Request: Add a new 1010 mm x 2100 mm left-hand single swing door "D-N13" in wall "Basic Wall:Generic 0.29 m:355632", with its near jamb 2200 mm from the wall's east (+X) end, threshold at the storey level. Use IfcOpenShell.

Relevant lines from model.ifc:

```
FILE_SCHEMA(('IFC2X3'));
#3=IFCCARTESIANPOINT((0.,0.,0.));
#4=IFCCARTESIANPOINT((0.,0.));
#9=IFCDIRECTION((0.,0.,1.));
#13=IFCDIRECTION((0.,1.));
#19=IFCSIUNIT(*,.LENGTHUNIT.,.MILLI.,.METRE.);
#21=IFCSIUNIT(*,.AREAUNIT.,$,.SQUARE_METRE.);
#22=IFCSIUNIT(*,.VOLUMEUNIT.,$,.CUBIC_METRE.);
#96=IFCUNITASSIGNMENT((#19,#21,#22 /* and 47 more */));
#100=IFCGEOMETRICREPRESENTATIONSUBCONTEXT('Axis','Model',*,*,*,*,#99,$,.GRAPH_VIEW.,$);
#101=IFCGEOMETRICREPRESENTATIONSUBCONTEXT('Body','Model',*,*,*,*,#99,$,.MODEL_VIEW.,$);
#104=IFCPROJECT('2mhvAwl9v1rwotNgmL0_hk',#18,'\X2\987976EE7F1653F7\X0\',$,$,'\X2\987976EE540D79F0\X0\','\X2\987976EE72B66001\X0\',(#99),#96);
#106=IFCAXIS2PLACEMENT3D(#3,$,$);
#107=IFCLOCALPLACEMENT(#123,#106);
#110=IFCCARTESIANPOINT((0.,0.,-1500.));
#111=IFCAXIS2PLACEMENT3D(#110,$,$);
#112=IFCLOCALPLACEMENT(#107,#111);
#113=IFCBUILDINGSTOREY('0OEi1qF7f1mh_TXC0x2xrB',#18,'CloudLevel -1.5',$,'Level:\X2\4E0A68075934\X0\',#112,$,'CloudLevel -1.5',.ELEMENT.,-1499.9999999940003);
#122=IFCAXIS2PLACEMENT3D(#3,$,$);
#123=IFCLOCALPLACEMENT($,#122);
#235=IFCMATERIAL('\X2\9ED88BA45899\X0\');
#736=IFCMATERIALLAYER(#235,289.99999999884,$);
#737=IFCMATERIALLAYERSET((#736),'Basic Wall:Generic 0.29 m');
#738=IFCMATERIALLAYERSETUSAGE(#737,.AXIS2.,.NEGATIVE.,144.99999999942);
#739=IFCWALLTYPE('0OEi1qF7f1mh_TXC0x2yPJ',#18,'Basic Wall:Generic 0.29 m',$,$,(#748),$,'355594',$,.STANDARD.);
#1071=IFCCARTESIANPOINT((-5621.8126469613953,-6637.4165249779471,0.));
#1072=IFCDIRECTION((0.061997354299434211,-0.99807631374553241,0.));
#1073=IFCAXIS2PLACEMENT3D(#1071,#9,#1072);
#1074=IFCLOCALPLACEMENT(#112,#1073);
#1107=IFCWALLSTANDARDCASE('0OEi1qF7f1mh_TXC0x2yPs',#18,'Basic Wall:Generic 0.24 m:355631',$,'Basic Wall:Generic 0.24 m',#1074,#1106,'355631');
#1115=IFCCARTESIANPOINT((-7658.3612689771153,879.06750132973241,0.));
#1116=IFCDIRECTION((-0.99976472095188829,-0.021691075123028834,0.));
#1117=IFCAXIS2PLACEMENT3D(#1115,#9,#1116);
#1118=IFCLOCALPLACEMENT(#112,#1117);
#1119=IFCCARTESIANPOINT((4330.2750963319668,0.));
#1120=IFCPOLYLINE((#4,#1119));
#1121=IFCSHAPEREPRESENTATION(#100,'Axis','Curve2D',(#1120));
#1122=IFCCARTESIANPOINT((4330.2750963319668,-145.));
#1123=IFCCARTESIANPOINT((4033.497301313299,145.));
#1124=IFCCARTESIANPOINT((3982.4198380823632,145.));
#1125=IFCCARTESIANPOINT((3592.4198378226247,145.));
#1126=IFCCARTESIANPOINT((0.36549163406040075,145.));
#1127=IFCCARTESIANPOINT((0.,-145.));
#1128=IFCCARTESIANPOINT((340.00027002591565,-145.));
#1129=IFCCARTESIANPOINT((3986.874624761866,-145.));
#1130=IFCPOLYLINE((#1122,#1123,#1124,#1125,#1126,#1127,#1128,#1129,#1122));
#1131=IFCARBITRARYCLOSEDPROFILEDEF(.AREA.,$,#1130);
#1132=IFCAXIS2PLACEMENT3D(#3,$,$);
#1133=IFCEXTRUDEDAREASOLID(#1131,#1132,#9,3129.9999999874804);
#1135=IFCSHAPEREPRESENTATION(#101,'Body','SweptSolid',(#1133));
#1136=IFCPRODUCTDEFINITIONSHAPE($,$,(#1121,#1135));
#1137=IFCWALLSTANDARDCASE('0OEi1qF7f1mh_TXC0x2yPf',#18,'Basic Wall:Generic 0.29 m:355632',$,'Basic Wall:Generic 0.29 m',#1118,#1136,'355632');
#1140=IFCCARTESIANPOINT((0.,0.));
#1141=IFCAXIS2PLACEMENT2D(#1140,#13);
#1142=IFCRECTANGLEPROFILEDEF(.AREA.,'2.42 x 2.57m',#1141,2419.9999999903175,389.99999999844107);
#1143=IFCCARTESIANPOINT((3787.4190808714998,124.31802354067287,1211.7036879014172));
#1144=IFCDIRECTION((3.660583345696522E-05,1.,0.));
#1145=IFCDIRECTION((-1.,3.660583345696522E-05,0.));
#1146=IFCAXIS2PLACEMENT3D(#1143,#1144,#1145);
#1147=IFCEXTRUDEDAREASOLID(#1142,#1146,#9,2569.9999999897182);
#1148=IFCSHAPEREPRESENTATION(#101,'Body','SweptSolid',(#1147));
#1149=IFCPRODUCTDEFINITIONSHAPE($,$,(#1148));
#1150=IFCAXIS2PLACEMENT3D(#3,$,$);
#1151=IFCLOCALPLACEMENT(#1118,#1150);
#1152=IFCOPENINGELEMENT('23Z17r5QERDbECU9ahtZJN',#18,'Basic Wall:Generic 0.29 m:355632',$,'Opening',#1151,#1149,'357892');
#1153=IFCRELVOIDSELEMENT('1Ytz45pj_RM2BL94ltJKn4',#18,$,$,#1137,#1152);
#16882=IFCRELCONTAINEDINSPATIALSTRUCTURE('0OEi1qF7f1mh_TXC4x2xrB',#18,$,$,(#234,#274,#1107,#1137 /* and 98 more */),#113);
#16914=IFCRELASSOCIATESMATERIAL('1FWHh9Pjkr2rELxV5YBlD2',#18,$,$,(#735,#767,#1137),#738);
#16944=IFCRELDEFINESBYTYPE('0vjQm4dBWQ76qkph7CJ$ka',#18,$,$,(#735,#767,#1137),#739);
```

```python
import numpy as np
import ifcopenshell
import ifcopenshell.api.feature
import ifcopenshell.api.geometry
import ifcopenshell.api.root
import ifcopenshell.api.spatial
import ifcopenshell.api.type
import ifcopenshell.geom
import ifcopenshell.util.element
import ifcopenshell.util.placement
import ifcopenshell.util.representation
import ifcopenshell.util.shape
import ifcopenshell.util.unit

model = ifcopenshell.open("model.ifc")
unit_scale = ifcopenshell.util.unit.calculate_unit_scale(model)
settings = ifcopenshell.geom.settings()


def volume(element):
    """Net volume in cubic metres, openings subtracted."""
    shape = ifcopenshell.geom.create_shape(settings, element)
    return ifcopenshell.util.shape.get_volume(shape.geometry)


wall = model.by_guid("0OEi1qF7f1mh_TXC0x2yPf")
storey = ifcopenshell.util.element.get_container(wall, ifc_class="IfcBuildingStorey")
context = ifcopenshell.util.representation.get_context(model, "Model", "Body", "MODEL_VIEW")
before = volume(wall)

width, height, from_end, sill = 1.01, 2.1, 2.2, 0.0  # metres

# The wall runs along its own X axis, and the end named is its -X end.
wall_shape = ifcopenshell.geom.create_shape(settings, wall)
x, y, z = ifcopenshell.util.shape.get_vertices(wall_shape.geometry).T
start = x.min() + from_end
face, thickness = float(y.min()), float(y.max() - y.min())
wall_matrix = ifcopenshell.util.placement.get_local_placement(wall.ObjectPlacement)
level = ifcopenshell.util.placement.get_local_placement(storey.ObjectPlacement)[2, 3]


def in_wall(x, y):
    """Placement at x, y metres in the wall's axes, at sill height."""
    matrix = wall_matrix.copy()
    matrix[:, 3] = wall_matrix @ np.array([x / unit_scale, y / unit_scale, 0.0, 1.0])
    matrix[2, 3] = level + sill / unit_scale
    return matrix


# Opening: a box that overshoots both wall faces by 50 mm.
opening = ifcopenshell.api.root.create_entity(model, ifc_class="IfcOpeningElement")
box = ifcopenshell.api.geometry.add_wall_representation(
    model, context=context, length=width, height=height, thickness=thickness + 0.1
)
ifcopenshell.api.geometry.assign_representation(model, product=opening, representation=box)
ifcopenshell.api.geometry.edit_object_placement(model, product=opening, matrix=in_wall(start, face - 0.05), is_si=False)
ifcopenshell.api.feature.add_feature(model, feature=opening, element=wall)

door = ifcopenshell.api.root.create_entity(model, ifc_class="IfcDoor", name="D-N13")
door.OverallWidth, door.OverallHeight = width / unit_scale, height / unit_scale
body = ifcopenshell.api.geometry.add_door_representation(
    model,
    context=context,
    overall_width=door.OverallWidth,
    overall_height=door.OverallHeight,
    operation_type="SINGLE_SWING_LEFT",
    lining_properties={"LiningDepth": thickness / unit_scale, "ThresholdDepth": thickness / unit_scale},
)
ifcopenshell.api.geometry.assign_representation(model, product=door, representation=body)
ifcopenshell.api.spatial.assign_container(model, products=[door], relating_structure=storey)
fills = ifcopenshell.api.feature.add_filling(model, opening=opening, element=door)
fills.OwnerHistory = door.OwnerHistory  # required in IFC2X3

# IFC2X3 keeps the operation on the door style.
style = ifcopenshell.api.root.create_entity(model, ifc_class="IfcDoorStyle", name="D-N13")
style.OperationType, style.ConstructionType = "SINGLE_SWING_LEFT", "NOTDEFINED"
style.ParameterTakesPrecedence = style.Sizeable = False
ifcopenshell.api.type.assign_type(model, related_objects=[door], relating_type=style)

# The lining spans the wall, so the door starts at the wall face.
ifcopenshell.api.geometry.edit_object_placement(model, product=door, matrix=in_wall(start, face), is_si=False)

after = volume(wall)

print(f"wall volume {before:.3f} -> {after:.3f} m3")

model.write("model_updated.ifc")
```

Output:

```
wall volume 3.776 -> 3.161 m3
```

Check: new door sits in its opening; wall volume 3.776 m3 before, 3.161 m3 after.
